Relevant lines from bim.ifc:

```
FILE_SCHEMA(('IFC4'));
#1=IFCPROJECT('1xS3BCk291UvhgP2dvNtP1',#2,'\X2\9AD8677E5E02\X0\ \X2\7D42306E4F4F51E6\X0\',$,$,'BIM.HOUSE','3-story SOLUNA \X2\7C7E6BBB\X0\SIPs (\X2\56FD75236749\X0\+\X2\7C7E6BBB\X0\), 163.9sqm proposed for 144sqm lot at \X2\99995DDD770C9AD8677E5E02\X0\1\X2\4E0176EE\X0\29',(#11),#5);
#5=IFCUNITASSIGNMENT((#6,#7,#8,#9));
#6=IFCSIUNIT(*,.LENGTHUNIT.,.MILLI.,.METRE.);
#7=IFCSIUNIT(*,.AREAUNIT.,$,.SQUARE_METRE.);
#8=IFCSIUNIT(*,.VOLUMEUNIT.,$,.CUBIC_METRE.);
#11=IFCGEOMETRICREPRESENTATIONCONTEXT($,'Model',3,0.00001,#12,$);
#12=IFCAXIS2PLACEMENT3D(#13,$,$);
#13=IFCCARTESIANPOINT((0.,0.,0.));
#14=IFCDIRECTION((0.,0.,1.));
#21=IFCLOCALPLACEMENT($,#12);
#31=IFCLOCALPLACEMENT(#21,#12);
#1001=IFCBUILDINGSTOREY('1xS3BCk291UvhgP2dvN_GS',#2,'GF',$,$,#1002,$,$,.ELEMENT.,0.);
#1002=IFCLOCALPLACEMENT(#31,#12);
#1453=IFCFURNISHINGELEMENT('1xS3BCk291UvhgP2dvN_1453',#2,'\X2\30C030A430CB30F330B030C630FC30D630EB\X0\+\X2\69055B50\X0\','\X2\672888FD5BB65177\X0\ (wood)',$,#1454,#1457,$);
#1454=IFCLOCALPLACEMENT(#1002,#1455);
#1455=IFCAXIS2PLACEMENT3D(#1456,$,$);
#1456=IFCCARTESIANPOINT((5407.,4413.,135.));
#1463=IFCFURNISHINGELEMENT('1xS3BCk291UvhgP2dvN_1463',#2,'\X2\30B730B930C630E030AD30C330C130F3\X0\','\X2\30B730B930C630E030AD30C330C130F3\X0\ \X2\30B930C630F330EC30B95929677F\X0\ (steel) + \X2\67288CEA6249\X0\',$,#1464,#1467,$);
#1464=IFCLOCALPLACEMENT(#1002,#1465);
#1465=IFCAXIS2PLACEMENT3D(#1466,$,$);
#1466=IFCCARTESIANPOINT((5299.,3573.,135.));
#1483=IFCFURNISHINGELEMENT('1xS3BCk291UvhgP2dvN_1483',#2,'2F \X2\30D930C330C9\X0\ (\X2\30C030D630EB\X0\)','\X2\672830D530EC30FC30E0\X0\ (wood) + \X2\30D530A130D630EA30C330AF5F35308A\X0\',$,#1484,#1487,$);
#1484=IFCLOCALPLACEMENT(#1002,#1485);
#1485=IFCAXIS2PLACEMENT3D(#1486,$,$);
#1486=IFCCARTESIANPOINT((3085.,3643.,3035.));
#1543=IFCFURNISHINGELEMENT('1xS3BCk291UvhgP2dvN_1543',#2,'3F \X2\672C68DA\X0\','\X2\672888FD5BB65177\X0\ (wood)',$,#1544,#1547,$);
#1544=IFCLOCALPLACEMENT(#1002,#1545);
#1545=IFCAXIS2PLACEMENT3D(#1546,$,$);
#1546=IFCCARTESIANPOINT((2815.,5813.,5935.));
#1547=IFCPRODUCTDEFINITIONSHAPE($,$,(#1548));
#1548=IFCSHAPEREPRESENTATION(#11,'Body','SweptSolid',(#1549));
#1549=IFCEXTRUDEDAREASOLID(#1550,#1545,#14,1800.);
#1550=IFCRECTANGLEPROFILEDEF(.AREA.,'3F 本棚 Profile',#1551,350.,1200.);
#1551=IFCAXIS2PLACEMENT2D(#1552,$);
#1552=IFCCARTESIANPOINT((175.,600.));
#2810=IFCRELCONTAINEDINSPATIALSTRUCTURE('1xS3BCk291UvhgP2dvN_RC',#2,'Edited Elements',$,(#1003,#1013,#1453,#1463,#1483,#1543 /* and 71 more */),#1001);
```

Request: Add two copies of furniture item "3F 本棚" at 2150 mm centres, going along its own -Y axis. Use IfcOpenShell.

```python
import ifcopenshell
import ifcopenshell.api.geometry
import ifcopenshell.api.root
import ifcopenshell.util.element
import ifcopenshell.util.placement
import ifcopenshell.util.unit

model = ifcopenshell.open("bim.ifc")
unit_scale = ifcopenshell.util.unit.calculate_unit_scale(model)


def reuse_history(source, copy):
    """copy_class also copies each property set's owner history, people and application; keep the originals."""
    for rel in copy.IsDefinedBy:
        if rel.is_a("IfcRelDefinesByProperties") and (history := rel.RelatingPropertyDefinition.OwnerHistory):
            rel.RelatingPropertyDefinition.OwnerHistory = source.OwnerHistory
            ifcopenshell.util.element.remove_deep2(model, history)


source = model.by_guid("1xS3BCk291UvhgP2dvN_1543")
base = ifcopenshell.util.placement.get_local_placement(source.ObjectPlacement)
step = -base[:3, 1] * 2.15 / unit_scale

for i in range(1, 3):
    copy = ifcopenshell.api.root.copy_class(model, product=source)
    copy.Representation = ifcopenshell.util.element.copy_deep(
        model, source.Representation, exclude=["IfcGeometricRepresentationContext", "IfcRepresentationMap"]
    )
    reuse_history(source, copy)
    matrix = base.copy()
    matrix[:3, 3] += i * step
    print("added at", matrix[:3, 3].round(3) + 0.0)
    ifcopenshell.api.geometry.edit_object_placement(model, product=copy, matrix=matrix, is_si=False)

model.write("bim_edited.ifc")
```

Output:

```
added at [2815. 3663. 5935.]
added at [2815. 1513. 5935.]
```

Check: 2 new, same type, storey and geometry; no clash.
